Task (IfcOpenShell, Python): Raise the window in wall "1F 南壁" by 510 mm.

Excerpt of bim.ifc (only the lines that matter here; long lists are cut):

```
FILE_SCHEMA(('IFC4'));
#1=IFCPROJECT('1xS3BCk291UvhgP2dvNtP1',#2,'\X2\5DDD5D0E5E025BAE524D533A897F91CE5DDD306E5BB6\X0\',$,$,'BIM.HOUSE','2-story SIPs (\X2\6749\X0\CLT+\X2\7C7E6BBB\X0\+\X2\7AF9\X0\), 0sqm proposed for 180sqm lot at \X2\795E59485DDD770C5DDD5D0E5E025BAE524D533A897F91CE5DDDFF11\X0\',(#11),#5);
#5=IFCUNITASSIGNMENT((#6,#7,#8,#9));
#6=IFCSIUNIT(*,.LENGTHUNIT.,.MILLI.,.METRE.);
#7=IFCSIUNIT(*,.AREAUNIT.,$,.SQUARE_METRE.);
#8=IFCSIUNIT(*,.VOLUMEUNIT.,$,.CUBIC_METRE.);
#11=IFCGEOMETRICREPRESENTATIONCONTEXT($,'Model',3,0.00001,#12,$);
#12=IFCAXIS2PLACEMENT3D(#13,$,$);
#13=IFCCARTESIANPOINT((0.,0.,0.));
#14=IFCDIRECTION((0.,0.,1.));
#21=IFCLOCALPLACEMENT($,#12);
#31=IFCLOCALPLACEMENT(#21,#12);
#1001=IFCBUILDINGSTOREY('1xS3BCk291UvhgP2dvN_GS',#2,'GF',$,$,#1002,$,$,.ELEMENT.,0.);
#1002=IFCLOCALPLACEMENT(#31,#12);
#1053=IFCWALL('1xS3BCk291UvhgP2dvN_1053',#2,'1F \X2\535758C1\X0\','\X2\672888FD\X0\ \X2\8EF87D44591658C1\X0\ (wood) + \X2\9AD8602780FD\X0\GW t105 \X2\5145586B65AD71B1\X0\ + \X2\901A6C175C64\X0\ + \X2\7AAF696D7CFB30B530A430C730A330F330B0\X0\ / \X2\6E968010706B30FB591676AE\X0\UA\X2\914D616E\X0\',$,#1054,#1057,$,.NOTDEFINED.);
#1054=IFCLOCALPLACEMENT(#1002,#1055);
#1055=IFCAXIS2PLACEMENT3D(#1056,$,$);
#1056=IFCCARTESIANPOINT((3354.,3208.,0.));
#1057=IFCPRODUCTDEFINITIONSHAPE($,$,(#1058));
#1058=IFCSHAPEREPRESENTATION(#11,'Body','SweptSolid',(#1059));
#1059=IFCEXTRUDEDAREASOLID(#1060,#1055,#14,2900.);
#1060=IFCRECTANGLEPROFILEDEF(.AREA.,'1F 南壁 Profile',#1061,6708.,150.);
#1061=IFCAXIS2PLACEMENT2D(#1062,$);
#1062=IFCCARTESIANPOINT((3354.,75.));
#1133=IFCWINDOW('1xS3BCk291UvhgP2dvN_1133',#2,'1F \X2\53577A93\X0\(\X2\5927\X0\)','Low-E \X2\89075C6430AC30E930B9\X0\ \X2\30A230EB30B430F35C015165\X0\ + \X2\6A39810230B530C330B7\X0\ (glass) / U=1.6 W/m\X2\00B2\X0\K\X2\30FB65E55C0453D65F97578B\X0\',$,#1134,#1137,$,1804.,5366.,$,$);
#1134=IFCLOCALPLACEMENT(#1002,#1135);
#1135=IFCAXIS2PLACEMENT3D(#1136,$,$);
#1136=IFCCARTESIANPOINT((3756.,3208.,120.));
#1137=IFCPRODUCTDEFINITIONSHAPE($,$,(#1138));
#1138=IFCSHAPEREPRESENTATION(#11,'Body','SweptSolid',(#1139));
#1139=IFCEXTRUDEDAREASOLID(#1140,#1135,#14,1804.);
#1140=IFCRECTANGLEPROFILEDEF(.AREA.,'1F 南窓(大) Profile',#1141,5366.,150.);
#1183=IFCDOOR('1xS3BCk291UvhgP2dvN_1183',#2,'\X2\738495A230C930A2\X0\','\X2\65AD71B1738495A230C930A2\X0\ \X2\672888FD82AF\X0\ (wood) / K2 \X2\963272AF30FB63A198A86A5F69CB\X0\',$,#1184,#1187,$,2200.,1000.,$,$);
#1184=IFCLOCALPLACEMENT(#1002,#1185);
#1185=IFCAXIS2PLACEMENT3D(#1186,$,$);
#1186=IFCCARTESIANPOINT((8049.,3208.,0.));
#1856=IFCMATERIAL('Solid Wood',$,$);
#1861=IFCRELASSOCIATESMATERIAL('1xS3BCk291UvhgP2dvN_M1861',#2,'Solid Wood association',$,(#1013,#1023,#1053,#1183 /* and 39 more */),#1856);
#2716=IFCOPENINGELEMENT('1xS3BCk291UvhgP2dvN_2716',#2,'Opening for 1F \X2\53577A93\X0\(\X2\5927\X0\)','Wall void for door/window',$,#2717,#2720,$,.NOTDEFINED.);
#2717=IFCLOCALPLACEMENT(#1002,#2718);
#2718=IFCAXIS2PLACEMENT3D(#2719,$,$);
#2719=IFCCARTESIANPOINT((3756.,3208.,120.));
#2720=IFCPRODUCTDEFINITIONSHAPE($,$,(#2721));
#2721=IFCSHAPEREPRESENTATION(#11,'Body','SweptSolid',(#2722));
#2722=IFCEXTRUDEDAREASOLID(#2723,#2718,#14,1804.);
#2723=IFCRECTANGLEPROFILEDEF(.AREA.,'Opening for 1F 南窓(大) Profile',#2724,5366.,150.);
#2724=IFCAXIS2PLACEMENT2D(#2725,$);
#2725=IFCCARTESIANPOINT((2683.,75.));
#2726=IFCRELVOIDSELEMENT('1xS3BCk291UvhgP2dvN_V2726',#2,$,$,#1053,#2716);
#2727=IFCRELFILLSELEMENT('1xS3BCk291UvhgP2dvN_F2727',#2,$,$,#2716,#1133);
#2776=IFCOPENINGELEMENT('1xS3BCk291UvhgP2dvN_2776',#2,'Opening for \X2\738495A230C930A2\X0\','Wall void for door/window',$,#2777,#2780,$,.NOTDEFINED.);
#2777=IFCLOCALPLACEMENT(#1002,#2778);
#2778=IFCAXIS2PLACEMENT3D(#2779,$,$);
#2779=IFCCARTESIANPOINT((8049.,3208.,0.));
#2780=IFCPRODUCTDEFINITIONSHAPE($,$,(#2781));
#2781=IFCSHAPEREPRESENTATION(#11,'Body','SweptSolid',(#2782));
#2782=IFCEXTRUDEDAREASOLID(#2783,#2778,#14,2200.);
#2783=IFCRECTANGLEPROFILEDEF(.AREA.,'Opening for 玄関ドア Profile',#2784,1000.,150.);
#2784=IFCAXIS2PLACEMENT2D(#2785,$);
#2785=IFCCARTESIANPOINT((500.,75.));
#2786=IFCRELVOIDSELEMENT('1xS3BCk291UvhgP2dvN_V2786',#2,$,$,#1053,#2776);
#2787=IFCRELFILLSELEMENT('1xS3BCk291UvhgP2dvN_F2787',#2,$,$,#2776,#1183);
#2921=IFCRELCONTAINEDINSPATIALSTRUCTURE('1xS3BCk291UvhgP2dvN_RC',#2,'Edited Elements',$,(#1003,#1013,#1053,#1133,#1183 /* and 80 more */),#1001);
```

```python
import numpy as np
import ifcopenshell
import ifcopenshell.api.geometry
import ifcopenshell.util.placement
import ifcopenshell.util.unit

model = ifcopenshell.open("bim.ifc")
unit_scale = ifcopenshell.util.unit.calculate_unit_scale(model)

window = model.by_guid("1xS3BCk291UvhgP2dvN_1133")
opening = window.FillsVoids[0].RelatingOpeningElement
dz = 510.0

shift = np.array([0.0, 0.0, dz])
# The window is not placed relative to its opening, so move both.
for product in (opening, window):
    matrix = ifcopenshell.util.placement.get_local_placement(product.ObjectPlacement)
    matrix[:3, 3] += shift
    ifcopenshell.api.geometry.edit_object_placement(model, product=product, matrix=matrix, is_si=False)

print(f"moved by {dz * unit_scale:+.3f} m")

model.write("bim_edited.ifc")
```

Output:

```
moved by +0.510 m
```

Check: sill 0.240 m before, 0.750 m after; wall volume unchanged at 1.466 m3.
